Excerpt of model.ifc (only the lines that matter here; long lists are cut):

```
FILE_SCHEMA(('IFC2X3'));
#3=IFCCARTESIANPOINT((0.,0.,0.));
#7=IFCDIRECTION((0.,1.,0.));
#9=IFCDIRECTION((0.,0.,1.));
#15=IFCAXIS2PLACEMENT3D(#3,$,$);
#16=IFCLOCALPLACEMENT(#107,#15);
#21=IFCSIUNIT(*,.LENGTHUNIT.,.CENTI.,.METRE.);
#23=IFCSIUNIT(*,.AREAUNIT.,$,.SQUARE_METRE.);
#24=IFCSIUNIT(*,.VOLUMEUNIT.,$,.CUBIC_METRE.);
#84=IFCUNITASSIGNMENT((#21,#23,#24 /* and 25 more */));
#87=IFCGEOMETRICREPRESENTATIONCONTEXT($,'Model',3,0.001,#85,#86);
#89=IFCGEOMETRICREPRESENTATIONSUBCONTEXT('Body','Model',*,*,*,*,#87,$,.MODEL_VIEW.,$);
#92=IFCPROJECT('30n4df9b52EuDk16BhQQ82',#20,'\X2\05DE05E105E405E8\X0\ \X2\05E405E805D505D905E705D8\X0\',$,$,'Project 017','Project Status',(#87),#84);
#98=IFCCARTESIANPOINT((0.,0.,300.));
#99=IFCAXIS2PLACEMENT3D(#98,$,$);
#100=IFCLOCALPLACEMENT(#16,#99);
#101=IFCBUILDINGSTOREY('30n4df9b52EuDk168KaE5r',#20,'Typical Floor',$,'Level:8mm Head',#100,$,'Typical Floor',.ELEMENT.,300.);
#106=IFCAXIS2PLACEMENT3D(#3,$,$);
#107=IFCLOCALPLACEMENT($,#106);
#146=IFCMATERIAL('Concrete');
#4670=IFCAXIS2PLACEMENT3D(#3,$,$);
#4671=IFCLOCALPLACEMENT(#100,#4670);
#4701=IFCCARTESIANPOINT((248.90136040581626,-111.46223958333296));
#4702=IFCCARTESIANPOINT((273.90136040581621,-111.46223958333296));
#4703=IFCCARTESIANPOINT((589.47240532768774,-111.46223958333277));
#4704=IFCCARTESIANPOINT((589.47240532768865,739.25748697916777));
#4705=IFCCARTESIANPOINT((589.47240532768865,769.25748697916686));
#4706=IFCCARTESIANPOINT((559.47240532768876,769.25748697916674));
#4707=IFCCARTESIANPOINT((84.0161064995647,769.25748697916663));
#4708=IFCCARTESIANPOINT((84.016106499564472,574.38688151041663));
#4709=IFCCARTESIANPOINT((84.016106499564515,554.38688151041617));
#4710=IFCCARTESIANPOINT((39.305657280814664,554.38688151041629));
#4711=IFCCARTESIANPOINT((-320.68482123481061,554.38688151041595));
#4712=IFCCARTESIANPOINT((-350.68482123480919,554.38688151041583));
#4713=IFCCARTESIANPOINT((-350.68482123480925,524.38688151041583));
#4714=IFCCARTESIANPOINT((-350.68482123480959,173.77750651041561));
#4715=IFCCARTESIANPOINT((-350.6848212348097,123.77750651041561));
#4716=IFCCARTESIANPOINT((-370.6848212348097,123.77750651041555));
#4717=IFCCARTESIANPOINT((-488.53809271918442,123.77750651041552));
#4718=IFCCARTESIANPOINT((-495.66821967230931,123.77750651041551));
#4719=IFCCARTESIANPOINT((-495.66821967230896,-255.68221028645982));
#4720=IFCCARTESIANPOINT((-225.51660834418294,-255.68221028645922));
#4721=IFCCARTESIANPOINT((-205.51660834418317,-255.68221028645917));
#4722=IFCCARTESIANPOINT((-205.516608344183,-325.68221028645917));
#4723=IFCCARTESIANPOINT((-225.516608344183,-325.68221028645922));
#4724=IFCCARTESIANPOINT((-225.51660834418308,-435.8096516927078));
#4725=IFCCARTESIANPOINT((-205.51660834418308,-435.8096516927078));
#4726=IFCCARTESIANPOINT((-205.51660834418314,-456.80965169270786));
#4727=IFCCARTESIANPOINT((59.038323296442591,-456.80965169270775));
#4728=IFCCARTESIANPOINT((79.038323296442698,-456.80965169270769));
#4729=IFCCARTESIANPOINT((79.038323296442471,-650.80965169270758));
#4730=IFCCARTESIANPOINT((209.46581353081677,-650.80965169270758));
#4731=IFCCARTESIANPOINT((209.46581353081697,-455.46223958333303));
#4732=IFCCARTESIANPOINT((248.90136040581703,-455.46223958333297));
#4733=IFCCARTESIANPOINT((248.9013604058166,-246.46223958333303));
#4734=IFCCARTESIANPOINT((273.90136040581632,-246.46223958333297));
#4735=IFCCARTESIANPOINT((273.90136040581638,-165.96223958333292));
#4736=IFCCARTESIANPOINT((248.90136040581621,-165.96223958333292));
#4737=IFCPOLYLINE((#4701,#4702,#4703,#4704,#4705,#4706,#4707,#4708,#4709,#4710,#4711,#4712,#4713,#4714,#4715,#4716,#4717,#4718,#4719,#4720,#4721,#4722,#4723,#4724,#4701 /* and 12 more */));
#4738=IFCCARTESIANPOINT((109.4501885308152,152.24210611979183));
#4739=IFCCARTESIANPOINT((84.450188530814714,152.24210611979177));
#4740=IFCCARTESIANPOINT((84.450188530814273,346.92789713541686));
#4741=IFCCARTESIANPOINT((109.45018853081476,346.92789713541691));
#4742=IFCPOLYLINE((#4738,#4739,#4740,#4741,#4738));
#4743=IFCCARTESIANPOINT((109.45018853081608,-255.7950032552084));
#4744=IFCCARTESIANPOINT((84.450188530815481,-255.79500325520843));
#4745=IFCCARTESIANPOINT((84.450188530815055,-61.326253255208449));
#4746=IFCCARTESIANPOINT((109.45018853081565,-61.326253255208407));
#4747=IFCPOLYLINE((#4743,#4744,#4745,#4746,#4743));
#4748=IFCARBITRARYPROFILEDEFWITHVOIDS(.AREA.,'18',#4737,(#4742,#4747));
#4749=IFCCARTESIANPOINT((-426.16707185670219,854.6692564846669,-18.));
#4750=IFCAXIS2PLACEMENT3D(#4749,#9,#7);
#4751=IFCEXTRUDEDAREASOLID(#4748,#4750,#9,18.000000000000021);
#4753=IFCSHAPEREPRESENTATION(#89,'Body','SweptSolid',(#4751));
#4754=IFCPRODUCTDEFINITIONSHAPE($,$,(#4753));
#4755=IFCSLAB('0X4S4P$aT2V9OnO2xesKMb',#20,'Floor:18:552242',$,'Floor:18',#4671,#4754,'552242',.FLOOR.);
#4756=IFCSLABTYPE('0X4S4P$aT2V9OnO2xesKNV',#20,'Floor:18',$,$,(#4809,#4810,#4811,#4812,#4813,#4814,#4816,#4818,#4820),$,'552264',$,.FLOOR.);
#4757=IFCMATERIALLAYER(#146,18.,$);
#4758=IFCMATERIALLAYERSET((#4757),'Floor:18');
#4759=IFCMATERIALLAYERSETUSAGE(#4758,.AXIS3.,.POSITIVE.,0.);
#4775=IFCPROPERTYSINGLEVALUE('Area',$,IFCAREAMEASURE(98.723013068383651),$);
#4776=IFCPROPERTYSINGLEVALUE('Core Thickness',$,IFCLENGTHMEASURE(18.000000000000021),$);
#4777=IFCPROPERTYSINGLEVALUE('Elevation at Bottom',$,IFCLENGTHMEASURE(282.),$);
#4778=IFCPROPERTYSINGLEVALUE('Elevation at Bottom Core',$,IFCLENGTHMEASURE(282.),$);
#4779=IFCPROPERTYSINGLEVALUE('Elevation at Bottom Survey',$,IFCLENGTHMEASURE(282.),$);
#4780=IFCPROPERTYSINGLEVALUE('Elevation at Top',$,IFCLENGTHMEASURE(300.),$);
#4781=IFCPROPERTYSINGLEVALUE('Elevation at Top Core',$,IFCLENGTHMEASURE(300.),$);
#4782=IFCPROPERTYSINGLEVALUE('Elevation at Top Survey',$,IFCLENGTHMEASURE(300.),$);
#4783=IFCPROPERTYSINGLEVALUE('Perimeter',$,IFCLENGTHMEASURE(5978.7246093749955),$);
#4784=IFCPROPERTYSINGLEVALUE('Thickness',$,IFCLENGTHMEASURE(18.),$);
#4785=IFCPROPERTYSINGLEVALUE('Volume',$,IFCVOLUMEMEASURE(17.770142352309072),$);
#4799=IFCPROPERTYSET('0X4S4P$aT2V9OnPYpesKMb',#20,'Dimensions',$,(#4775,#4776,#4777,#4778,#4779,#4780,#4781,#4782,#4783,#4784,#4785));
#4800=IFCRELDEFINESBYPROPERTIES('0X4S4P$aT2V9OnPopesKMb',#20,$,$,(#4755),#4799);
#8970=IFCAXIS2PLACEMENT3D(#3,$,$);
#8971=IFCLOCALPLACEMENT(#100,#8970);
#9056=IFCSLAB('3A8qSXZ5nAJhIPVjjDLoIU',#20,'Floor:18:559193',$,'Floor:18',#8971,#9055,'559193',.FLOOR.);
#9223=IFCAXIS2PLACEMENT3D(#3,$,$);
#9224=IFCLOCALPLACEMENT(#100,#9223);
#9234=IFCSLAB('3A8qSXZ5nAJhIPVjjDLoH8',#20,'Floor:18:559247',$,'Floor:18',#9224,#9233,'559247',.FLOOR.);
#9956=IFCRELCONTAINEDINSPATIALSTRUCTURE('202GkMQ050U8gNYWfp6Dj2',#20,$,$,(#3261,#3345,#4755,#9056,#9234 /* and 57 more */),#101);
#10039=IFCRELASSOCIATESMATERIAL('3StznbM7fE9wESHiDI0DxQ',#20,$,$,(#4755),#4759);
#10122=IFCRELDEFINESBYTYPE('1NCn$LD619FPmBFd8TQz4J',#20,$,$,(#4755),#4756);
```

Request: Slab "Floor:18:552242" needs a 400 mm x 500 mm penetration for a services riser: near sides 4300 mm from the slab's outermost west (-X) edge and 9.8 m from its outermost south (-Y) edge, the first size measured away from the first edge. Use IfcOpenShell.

```python
import numpy as np
import ifcopenshell
import ifcopenshell.api.feature
import ifcopenshell.api.geometry
import ifcopenshell.api.pset
import ifcopenshell.api.root
import ifcopenshell.geom
import ifcopenshell.util.element
import ifcopenshell.util.placement
import ifcopenshell.util.representation
import ifcopenshell.util.shape
import ifcopenshell.util.unit

model = ifcopenshell.open("model.ifc")
unit_scale = ifcopenshell.util.unit.calculate_unit_scale(model)
area_scale = ifcopenshell.util.unit.calculate_unit_scale(model, "AREAUNIT")
volume_scale = ifcopenshell.util.unit.calculate_unit_scale(model, "VOLUMEUNIT")
settings = ifcopenshell.geom.settings()


def volume(element):
    """Net volume in cubic metres, openings subtracted."""
    shape = ifcopenshell.geom.create_shape(settings, element)
    return ifcopenshell.util.shape.get_volume(shape.geometry)


slab = model.by_guid("0X4S4P$aT2V9OnO2xesKMb")
before = volume(slab)

# Extent in the slab's own axes, in metres. The edges named are its -X and -Y sides.
slab_shape = ifcopenshell.geom.create_shape(settings, slab)
vertices = ifcopenshell.util.shape.get_vertices(slab_shape.geometry)
x_min, y_min, bottom = vertices.min(axis=0)
top = vertices[:, 2].max()

opening = ifcopenshell.api.root.create_entity(model, ifc_class="IfcOpeningElement", name="Services riser opening")
context = ifcopenshell.util.representation.get_context(model, "Model", "Body", "MODEL_VIEW")
width, depth = 0.4, 0.5
outline = [(0.0, 0.0), (width, 0.0), (width, depth), (0.0, depth), (0.0, 0.0)]
# Overshoot both faces by 50 mm so the cut is clean.
shape = ifcopenshell.api.geometry.add_slab_representation(
    model, context=context, depth=top - bottom + 0.1, polyline=outline
)
ifcopenshell.api.geometry.assign_representation(model, product=opening, representation=shape)

matrix = ifcopenshell.util.placement.get_local_placement(slab.ObjectPlacement)
matrix[:, 3] = matrix @ np.append(np.array([x_min + 4.3, y_min + 9.8, bottom - 0.05]) / unit_scale, 1.0)
ifcopenshell.api.geometry.edit_object_placement(model, product=opening, matrix=matrix, is_si=False)
ifcopenshell.api.feature.add_feature(model, feature=opening, element=slab)

after = volume(slab)

# Update the slab's stored quantities.
pset = model.by_id(ifcopenshell.util.element.get_pset(slab, "Dimensions", should_inherit=False)["id"])
ifcopenshell.api.pset.edit_pset(model, pset=pset, properties={
    "Area": model.create_entity("IfcAreaMeasure", after / (top - bottom) / area_scale),
    "Volume": model.create_entity("IfcVolumeMeasure", after / volume_scale),
})

print(f"slab volume {before:.3f} -> {after:.3f} m3")

model.write("model_rev.ifc")
```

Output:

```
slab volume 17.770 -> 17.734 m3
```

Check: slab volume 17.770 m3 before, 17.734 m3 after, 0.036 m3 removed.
